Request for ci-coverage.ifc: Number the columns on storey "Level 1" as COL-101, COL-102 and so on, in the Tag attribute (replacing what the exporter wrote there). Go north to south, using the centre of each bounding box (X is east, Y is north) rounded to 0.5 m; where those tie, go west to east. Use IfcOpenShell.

First a look at what the model holds.

```python
import ifcopenshell
import ifcopenshell.util.element
import ifcopenshell.util.placement

model = ifcopenshell.open("ci-coverage.ifc")
print(model.schema)
storey = next(s for s in model.by_type("IfcBuildingStorey") if s.Name == "Level 1")
columns = [e for e in ifcopenshell.util.element.get_decomposition(storey) if e.is_a("IfcColumn")]
for e in sorted(columns, key=lambda e: e.id()):
    origin = ifcopenshell.util.placement.get_local_placement(e.ObjectPlacement)[:3, 3]
    print(e.id(), e.Tag, e.Name, origin.round(2) + 0.0, sep=" | ")
```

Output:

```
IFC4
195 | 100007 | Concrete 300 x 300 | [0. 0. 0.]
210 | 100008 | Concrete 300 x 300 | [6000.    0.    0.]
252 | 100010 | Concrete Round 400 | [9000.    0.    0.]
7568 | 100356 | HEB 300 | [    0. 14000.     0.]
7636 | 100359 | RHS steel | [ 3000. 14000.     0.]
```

```python
import ifcopenshell
import ifcopenshell.geom
import ifcopenshell.util.element
import ifcopenshell.util.shape

model = ifcopenshell.open("ci-coverage.ifc")
settings = ifcopenshell.geom.settings()
settings.set("use-world-coords", True)


def centre(element):
    shape = ifcopenshell.geom.create_shape(settings, element)
    return ifcopenshell.util.shape.get_bbox_centroid(shape.geometry)


storey = next(s for s in model.by_type("IfcBuildingStorey") if s.Name == "Level 1")
columns = [e for e in ifcopenshell.util.element.get_decomposition(storey) if e.is_a("IfcColumn")]

# Insertion points can sit at a corner or the storey origin, so sort by the geometry (in metres).
centres = {e: centre(e) for e in columns}
columns.sort(key=lambda e: (-round(centres[e][1] / 0.5), centres[e][0]))

for i, e in enumerate(columns, start=1):
    number = f"COL-1{i:02d}"
    e.Tag = number
    print(e.id(), number)

model.write("ci-coverage_v2.ifc")
```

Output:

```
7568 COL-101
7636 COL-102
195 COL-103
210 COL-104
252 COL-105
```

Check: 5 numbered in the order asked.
